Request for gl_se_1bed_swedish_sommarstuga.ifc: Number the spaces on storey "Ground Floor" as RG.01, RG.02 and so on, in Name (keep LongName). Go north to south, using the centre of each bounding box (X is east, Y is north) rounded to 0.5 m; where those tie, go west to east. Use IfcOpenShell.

First a look at what the model holds.

```python
import ifcopenshell
import ifcopenshell.util.element
import ifcopenshell.util.placement

model = ifcopenshell.open("gl_se_1bed_swedish_sommarstuga.ifc")
print(model.schema)
storey = next(s for s in model.by_type("IfcBuildingStorey") if s.Name == "Ground Floor")
spaces = [e for e in ifcopenshell.util.element.get_decomposition(storey) if e.is_a("IfcSpace")]
for e in sorted(spaces, key=lambda e: e.id()):
    origin = ifcopenshell.util.placement.get_local_placement(e.ObjectPlacement)[:3, 3]
    print(e.id(), e.Name, e.LongName, origin.round(2) + 0.0, sep=" | ")
```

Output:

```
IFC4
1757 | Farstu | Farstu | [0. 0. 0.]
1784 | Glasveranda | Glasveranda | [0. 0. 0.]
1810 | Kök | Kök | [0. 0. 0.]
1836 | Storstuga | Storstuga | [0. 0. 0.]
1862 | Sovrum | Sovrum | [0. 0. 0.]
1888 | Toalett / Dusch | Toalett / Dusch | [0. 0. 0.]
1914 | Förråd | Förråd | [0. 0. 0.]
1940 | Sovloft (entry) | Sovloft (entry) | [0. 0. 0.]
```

```python
import ifcopenshell
import ifcopenshell.geom
import ifcopenshell.util.element
import ifcopenshell.util.shape

model = ifcopenshell.open("gl_se_1bed_swedish_sommarstuga.ifc")
settings = ifcopenshell.geom.settings()
settings.set("use-world-coords", True)


def centre(element):
    shape = ifcopenshell.geom.create_shape(settings, element)
    return ifcopenshell.util.shape.get_bbox_centroid(shape.geometry)


storey = next(s for s in model.by_type("IfcBuildingStorey") if s.Name == "Ground Floor")
spaces = [e for e in ifcopenshell.util.element.get_decomposition(storey) if e.is_a("IfcSpace")]

# Insertion points can sit at a corner or the storey origin, so sort by the geometry (in metres).
centres = {e: centre(e) for e in spaces}
spaces.sort(key=lambda e: (-round(centres[e][1] / 0.5), centres[e][0]))

for i, e in enumerate(spaces, start=1):
    number = f"RG.{i:02d}"
    e.Name = number
    print(e.id(), number)

model.write("gl_se_1bed_swedish_sommarstuga-out.ifc")
```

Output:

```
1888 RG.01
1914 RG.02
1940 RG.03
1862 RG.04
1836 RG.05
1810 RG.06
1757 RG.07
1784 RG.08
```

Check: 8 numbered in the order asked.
